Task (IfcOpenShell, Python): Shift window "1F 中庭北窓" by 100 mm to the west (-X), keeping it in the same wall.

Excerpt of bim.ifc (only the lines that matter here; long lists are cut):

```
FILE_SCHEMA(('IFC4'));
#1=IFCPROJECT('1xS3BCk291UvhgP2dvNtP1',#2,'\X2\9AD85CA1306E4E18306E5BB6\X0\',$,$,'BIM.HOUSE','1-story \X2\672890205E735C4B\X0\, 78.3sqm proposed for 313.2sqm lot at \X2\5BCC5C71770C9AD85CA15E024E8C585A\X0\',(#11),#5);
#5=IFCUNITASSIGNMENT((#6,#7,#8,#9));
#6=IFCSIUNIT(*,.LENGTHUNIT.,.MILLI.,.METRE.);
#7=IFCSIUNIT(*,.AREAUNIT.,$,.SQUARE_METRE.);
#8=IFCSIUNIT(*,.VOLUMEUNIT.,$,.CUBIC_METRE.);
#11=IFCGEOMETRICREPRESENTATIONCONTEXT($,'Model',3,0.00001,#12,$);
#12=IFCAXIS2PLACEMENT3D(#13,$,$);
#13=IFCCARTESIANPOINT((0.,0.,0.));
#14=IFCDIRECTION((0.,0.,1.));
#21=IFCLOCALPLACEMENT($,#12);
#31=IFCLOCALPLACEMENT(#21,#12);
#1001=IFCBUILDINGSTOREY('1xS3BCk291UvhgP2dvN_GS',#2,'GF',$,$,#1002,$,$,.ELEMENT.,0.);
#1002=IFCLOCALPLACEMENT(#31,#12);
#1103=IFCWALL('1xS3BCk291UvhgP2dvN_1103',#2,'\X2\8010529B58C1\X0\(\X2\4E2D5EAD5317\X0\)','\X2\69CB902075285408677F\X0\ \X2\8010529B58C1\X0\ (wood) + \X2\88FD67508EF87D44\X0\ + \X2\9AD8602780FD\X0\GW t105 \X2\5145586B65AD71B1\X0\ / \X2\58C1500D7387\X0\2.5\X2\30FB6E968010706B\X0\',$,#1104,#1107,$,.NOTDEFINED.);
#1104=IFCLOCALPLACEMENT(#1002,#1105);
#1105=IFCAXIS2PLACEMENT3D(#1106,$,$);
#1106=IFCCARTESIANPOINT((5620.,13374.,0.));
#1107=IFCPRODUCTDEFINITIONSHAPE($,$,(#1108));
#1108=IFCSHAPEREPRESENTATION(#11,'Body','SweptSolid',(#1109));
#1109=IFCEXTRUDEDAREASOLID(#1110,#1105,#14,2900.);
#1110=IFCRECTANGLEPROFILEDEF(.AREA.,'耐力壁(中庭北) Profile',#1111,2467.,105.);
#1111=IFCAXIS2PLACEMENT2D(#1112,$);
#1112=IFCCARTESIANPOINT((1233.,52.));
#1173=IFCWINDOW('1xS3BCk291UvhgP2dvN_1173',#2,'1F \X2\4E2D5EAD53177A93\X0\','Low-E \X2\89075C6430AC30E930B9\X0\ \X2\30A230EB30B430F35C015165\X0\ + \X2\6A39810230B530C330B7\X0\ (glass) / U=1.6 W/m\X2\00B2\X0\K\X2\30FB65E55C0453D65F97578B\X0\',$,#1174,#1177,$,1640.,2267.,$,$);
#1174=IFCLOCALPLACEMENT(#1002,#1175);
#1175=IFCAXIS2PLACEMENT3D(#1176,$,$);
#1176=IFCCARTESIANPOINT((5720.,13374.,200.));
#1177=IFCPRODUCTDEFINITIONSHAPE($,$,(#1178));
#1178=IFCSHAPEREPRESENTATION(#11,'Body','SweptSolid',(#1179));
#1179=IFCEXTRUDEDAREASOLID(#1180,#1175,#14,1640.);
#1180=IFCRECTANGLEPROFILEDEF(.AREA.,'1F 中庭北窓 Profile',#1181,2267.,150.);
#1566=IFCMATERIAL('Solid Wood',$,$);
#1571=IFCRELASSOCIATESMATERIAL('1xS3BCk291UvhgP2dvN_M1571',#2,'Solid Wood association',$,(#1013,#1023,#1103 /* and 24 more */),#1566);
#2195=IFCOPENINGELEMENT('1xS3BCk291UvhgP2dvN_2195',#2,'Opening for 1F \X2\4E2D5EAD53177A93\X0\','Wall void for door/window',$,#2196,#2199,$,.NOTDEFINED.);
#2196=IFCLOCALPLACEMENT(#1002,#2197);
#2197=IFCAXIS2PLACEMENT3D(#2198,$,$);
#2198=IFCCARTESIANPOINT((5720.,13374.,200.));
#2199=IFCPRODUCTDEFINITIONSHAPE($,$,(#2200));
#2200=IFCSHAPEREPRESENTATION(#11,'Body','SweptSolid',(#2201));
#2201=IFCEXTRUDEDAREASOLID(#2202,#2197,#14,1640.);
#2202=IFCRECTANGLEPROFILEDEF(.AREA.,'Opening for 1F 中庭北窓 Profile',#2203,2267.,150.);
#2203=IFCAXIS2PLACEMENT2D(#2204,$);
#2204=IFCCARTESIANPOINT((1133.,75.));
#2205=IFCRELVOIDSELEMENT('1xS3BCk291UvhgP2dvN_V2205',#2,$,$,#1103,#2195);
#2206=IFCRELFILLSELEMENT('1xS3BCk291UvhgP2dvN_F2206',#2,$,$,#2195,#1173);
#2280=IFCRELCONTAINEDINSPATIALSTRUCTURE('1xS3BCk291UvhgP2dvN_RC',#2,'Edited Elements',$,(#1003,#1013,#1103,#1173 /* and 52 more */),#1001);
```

```python
import ifcopenshell
import ifcopenshell.api.geometry
import ifcopenshell.util.placement
import ifcopenshell.util.unit

model = ifcopenshell.open("bim.ifc")
unit_scale = ifcopenshell.util.unit.calculate_unit_scale(model)

window = model.by_guid("1xS3BCk291UvhgP2dvN_1173")
opening = window.FillsVoids[0].RelatingOpeningElement
wall = opening.VoidsElements[0].RelatingBuildingElement

wall_matrix = ifcopenshell.util.placement.get_local_placement(wall.ObjectPlacement)
shift = wall_matrix[:3, 0] * -0.1 / unit_scale
before = ifcopenshell.util.placement.get_local_placement(window.ObjectPlacement)[:3, 3].copy()

# The window is not placed relative to its opening, so move both.
for product in (opening, window):
    matrix = ifcopenshell.util.placement.get_local_placement(product.ObjectPlacement)
    matrix[:3, 3] += shift
    ifcopenshell.api.geometry.edit_object_placement(model, product=product, matrix=matrix, is_si=False)

after = ifcopenshell.util.placement.get_local_placement(window.ObjectPlacement)[:3, 3]
print("window moved by", (after - before).round(3) + 0.0)

model.write("bim_updated.ifc")
```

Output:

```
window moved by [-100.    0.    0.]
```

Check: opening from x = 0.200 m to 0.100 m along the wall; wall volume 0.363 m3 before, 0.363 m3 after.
